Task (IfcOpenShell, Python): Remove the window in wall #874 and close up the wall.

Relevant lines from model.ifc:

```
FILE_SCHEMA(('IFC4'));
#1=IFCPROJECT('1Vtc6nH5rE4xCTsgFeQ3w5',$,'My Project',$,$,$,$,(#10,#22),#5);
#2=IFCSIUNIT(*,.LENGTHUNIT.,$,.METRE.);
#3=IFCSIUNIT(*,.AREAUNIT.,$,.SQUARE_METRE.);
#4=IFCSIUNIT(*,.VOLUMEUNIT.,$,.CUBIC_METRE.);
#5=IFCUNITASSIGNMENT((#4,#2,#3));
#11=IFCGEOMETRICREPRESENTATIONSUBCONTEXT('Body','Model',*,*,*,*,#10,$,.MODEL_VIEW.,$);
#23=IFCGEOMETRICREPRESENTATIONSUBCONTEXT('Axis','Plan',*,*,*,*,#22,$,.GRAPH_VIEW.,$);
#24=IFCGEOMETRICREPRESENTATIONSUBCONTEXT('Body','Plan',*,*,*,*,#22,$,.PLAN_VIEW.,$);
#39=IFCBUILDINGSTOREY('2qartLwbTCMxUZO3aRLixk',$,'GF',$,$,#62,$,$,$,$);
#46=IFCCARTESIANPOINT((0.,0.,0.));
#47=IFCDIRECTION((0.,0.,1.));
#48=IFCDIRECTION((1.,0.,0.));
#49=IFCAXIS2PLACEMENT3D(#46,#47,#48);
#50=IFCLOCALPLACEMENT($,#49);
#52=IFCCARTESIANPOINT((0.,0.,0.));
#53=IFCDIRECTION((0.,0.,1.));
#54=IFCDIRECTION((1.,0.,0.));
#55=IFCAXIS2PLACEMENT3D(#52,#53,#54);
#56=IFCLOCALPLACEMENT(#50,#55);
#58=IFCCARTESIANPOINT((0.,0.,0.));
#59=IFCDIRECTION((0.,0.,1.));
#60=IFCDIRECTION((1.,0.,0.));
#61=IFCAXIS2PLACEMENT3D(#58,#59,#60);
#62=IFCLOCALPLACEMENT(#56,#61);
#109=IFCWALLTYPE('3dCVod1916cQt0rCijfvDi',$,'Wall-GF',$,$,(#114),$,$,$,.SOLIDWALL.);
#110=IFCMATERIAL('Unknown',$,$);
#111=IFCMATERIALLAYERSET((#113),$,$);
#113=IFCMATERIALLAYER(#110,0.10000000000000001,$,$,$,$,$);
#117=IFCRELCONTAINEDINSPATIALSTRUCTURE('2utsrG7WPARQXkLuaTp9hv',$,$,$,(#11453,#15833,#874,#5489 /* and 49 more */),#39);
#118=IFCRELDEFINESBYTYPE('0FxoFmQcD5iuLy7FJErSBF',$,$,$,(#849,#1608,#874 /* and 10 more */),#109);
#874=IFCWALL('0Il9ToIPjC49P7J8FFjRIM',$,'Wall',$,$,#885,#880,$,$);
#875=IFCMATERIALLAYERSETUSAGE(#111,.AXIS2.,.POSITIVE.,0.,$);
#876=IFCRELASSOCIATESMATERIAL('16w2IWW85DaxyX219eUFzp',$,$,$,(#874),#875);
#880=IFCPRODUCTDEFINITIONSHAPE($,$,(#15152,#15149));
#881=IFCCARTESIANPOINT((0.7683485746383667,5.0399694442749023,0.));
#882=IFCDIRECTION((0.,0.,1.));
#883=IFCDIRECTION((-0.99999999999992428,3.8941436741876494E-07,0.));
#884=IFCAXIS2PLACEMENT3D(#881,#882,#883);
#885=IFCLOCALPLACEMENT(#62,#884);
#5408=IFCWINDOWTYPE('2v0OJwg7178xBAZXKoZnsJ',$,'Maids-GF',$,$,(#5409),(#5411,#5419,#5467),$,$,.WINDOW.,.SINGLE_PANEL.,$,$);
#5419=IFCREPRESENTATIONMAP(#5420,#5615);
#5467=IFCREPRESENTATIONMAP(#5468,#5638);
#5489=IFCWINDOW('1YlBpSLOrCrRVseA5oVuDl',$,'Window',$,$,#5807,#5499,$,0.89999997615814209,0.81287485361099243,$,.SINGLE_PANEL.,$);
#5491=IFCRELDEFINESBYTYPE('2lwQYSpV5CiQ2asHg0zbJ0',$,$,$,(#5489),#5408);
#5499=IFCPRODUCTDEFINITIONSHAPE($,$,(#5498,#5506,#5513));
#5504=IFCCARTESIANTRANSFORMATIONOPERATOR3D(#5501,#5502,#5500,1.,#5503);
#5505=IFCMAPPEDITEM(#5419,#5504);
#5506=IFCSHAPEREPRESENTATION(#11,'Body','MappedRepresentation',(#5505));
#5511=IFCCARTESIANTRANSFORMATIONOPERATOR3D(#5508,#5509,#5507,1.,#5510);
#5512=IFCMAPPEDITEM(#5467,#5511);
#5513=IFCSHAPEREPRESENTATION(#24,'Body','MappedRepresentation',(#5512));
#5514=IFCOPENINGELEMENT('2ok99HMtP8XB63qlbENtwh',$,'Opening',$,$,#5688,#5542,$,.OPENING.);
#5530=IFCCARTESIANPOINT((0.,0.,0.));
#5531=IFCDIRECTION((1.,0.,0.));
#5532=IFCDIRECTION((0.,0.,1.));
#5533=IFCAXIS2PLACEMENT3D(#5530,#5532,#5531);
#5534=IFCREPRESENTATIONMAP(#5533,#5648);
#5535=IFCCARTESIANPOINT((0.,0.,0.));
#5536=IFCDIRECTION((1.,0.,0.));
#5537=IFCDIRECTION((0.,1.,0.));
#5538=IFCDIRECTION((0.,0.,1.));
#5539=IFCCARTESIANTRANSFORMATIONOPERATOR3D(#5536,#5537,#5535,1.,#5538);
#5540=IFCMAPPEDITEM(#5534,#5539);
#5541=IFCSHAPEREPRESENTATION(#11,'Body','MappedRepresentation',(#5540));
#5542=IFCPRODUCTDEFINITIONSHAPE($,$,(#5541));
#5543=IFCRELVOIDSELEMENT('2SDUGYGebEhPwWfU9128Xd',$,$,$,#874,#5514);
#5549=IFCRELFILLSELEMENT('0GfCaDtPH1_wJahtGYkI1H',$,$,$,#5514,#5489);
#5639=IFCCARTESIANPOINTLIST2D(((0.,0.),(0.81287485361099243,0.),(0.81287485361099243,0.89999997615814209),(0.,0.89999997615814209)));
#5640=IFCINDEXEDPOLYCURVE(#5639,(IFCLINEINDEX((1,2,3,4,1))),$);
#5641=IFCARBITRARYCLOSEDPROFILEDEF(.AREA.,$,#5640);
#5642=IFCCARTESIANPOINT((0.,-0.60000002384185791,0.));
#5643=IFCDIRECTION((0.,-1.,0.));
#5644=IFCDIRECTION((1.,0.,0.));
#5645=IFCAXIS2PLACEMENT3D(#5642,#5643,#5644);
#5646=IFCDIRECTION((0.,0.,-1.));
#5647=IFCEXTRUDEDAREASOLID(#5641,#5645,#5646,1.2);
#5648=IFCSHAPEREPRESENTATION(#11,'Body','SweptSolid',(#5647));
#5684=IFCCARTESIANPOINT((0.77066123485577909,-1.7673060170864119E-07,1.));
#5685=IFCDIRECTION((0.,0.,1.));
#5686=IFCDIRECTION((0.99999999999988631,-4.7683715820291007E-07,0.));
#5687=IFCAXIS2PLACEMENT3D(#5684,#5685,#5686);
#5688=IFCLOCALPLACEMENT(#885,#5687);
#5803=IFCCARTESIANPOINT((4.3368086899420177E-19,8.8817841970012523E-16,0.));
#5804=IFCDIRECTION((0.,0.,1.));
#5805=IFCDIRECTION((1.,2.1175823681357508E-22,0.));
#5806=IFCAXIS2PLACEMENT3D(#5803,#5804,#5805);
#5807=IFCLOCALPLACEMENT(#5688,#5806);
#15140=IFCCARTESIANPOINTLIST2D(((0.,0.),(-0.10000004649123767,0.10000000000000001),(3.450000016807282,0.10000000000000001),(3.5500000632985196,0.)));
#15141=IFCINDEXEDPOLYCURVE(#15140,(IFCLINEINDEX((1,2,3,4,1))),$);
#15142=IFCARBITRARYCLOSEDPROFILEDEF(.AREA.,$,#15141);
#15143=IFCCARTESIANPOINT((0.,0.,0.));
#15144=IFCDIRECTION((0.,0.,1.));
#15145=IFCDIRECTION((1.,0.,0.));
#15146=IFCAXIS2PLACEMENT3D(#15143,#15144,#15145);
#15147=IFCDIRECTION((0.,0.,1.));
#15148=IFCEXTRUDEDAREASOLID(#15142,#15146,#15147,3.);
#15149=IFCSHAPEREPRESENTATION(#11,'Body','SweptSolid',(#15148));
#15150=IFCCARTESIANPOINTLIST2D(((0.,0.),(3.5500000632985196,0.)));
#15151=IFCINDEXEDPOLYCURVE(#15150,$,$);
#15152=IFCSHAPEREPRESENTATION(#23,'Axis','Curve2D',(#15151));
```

```python
import ifcopenshell
import ifcopenshell.api.feature
import ifcopenshell.api.root
import ifcopenshell.geom
import ifcopenshell.util.shape

model = ifcopenshell.open("model.ifc")
settings = ifcopenshell.geom.settings()


def volume(element):
    """Net volume in cubic metres, openings subtracted."""
    shape = ifcopenshell.geom.create_shape(settings, element)
    return ifcopenshell.util.shape.get_volume(shape.geometry)


window = model.by_guid("1YlBpSLOrCrRVseA5oVuDl")
opening = window.FillsVoids[0].RelatingOpeningElement
wall = opening.VoidsElements[0].RelatingBuildingElement
before = volume(wall)

ifcopenshell.api.root.remove_product(model, product=window)
ifcopenshell.api.feature.remove_feature(model, feature=opening)

after = volume(wall)

print(f"wall volume {before:.3f} -> {after:.3f} m3")

model.write("model_v2.ifc")
```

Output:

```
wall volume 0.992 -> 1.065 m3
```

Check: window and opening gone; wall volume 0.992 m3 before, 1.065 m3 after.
